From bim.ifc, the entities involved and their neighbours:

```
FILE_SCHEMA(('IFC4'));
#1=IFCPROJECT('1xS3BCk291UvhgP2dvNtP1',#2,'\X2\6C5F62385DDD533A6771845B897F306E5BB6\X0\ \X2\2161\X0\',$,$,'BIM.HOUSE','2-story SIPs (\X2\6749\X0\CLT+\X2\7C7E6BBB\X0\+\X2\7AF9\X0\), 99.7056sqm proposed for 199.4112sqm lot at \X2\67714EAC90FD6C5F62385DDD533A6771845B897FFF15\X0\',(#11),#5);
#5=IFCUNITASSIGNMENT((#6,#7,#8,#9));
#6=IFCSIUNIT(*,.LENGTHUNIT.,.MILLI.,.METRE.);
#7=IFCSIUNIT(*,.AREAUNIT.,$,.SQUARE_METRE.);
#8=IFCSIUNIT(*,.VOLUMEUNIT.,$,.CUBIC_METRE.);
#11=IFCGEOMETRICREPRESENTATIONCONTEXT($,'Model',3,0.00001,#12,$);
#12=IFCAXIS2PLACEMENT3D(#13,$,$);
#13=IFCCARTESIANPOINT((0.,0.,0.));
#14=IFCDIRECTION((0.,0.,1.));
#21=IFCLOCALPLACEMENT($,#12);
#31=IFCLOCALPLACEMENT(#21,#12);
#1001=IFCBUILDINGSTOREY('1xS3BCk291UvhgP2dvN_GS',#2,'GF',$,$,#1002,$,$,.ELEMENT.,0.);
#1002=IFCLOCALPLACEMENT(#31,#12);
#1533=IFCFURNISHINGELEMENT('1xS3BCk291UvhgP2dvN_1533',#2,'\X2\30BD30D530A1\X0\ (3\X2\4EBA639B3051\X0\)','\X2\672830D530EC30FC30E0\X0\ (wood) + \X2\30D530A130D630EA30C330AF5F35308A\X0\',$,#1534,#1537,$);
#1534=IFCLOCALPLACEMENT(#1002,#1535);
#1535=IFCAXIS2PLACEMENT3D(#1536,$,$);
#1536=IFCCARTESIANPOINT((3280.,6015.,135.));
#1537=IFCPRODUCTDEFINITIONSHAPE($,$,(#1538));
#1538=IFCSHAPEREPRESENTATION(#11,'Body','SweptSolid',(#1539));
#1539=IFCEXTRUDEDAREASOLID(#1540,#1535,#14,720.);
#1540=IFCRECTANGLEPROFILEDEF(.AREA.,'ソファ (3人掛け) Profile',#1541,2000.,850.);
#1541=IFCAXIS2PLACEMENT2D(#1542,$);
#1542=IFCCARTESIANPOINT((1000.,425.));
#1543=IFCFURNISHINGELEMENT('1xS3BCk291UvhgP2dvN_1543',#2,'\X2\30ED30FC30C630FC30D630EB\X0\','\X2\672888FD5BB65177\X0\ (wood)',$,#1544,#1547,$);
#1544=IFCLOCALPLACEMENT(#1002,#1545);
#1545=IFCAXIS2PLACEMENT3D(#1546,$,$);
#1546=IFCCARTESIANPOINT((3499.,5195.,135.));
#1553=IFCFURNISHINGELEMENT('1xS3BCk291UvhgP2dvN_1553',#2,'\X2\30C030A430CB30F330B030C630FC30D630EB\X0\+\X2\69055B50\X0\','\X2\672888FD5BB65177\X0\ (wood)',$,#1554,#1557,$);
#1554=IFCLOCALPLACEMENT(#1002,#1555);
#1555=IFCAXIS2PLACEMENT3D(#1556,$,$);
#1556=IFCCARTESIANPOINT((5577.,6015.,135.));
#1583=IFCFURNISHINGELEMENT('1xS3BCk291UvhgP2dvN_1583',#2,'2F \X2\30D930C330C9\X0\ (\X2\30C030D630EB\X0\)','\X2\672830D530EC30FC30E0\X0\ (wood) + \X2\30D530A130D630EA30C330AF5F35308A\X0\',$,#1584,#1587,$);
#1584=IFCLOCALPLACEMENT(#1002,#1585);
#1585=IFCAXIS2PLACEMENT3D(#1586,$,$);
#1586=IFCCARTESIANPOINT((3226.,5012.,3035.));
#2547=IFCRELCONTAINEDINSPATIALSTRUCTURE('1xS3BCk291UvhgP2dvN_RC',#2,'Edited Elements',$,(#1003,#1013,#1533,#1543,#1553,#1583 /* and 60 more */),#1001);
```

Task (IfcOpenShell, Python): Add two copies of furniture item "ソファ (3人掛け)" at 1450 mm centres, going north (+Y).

```python
import numpy as np
import ifcopenshell
import ifcopenshell.api.geometry
import ifcopenshell.api.root
import ifcopenshell.util.element
import ifcopenshell.util.placement

model = ifcopenshell.open("bim.ifc")


def reuse_history(source, copy):
    """copy_class also copies each property set's owner history, people and application; keep the originals."""
    for rel in copy.IsDefinedBy:
        if rel.is_a("IfcRelDefinesByProperties") and (history := rel.RelatingPropertyDefinition.OwnerHistory):
            rel.RelatingPropertyDefinition.OwnerHistory = source.OwnerHistory
            ifcopenshell.util.element.remove_deep2(model, history)


source = model.by_guid("1xS3BCk291UvhgP2dvN_1533")
base = ifcopenshell.util.placement.get_local_placement(source.ObjectPlacement)
step = np.array([0.0, 1.0, 0.0]) * 1450.0

for i in range(1, 3):
    copy = ifcopenshell.api.root.copy_class(model, product=source)
    copy.Representation = ifcopenshell.util.element.copy_deep(
        model, source.Representation, exclude=["IfcGeometricRepresentationContext", "IfcRepresentationMap"]
    )
    reuse_history(source, copy)
    matrix = base.copy()
    matrix[:3, 3] += i * step
    print("added at", matrix[:3, 3].round(3) + 0.0)
    ifcopenshell.api.geometry.edit_object_placement(model, product=copy, matrix=matrix, is_si=False)

model.write("bim_v2.ifc")
```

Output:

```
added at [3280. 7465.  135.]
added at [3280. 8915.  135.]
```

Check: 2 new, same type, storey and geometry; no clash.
